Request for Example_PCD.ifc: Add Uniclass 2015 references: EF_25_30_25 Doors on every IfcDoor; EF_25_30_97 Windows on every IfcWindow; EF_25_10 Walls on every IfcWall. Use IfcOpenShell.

First a look at what the model holds.

```python
import ifcopenshell

model = ifcopenshell.open("Example_PCD.ifc")
print(model.schema)
print("classifications:", [c.Name for c in model.by_type("IfcClassification")])
for ifc_class in ("IfcDoor", "IfcRoof", "IfcStair", "IfcWall", "IfcWindow"):
    print(ifc_class, len(model.by_type(ifc_class)))
```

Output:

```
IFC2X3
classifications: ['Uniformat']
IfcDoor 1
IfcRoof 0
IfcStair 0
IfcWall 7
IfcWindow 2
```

```python
import ifcopenshell
import ifcopenshell.api.classification

model = ifcopenshell.open("Example_PCD.ifc")

# IFC2X3 requires Source and Edition and has no link from the project to the system.
system = model.create_entity("IfcClassification", Source="NBS", Edition="2015", Name="Uniclass 2015")

codes = {
    "IfcDoor": ("EF_25_30_25", "Doors"),
    "IfcWindow": ("EF_25_30_97", "Windows"),
    "IfcWall": ("EF_25_10", "Walls"),
}
for ifc_class, (code, name) in codes.items():
    products = model.by_type(ifc_class)
    ifcopenshell.api.classification.add_reference(
        model, products=products, classification=system, identification=code, name=name
    )
    print(code, len(products))

model.write("Example_PCD-out.ifc")
```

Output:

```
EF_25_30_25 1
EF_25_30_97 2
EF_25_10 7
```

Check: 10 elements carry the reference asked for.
